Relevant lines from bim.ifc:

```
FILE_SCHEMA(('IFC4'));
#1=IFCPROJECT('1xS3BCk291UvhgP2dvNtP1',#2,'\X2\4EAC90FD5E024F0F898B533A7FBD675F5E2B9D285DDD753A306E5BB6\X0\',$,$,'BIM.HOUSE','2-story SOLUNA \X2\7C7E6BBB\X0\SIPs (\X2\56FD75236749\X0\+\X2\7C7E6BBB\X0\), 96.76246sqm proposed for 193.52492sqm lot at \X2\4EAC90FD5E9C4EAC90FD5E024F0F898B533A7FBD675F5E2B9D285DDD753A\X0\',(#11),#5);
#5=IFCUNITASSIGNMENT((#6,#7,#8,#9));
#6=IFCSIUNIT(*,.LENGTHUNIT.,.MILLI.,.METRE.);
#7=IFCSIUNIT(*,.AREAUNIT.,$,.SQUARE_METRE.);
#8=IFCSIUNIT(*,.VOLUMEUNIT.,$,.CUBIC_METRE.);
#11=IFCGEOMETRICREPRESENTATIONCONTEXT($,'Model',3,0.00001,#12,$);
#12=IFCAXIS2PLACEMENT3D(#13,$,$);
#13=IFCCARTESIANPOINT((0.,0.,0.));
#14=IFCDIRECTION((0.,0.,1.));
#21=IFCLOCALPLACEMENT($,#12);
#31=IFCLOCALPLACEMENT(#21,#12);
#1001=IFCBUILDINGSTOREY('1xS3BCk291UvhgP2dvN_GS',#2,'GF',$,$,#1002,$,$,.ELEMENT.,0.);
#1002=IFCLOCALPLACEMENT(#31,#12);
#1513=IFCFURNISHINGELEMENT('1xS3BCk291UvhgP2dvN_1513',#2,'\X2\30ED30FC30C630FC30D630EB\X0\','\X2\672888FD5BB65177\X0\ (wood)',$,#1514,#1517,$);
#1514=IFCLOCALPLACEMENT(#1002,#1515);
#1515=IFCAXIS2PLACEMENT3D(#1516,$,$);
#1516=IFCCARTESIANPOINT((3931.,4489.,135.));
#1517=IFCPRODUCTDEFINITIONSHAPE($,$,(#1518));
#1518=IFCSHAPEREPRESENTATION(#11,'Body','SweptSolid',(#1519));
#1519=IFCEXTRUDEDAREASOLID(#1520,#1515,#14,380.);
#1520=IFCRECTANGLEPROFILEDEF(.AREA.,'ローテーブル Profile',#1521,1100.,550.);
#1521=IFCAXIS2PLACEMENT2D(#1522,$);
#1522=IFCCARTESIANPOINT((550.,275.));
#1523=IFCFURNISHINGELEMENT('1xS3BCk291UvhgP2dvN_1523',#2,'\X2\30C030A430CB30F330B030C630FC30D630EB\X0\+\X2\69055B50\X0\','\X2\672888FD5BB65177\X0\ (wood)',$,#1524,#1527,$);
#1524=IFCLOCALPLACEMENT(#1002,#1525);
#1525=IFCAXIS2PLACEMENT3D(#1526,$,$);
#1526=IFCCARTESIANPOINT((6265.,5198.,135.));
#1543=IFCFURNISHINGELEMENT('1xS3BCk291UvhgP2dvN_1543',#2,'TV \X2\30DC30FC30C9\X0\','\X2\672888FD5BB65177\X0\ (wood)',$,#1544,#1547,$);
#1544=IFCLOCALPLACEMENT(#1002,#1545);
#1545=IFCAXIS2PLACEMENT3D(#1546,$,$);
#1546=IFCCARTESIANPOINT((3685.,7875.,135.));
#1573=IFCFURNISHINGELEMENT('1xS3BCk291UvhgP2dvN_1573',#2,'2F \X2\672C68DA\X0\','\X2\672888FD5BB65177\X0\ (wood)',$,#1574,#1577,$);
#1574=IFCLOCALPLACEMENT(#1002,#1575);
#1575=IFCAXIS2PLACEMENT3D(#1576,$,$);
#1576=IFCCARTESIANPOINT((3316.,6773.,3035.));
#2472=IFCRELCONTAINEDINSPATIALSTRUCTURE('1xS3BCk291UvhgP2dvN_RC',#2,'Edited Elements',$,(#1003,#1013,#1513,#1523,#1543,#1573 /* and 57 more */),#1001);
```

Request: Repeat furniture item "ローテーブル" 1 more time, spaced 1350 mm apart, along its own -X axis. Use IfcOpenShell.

```python
import ifcopenshell
import ifcopenshell.api.geometry
import ifcopenshell.api.root
import ifcopenshell.util.element
import ifcopenshell.util.placement

model = ifcopenshell.open("bim.ifc")


def reuse_history(source, copy):
    """copy_class also copies each property set's owner history, people and application; keep the originals."""
    for rel in copy.IsDefinedBy:
        if rel.is_a("IfcRelDefinesByProperties") and (history := rel.RelatingPropertyDefinition.OwnerHistory):
            rel.RelatingPropertyDefinition.OwnerHistory = source.OwnerHistory
            ifcopenshell.util.element.remove_deep2(model, history)


source = model.by_guid("1xS3BCk291UvhgP2dvN_1513")
base = ifcopenshell.util.placement.get_local_placement(source.ObjectPlacement)
step = -base[:3, 0] * 1350.0

for i in range(1, 2):
    copy = ifcopenshell.api.root.copy_class(model, product=source)
    copy.Representation = ifcopenshell.util.element.copy_deep(
        model, source.Representation, exclude=["IfcGeometricRepresentationContext", "IfcRepresentationMap"]
    )
    reuse_history(source, copy)
    matrix = base.copy()
    matrix[:3, 3] += i * step
    print("added at", matrix[:3, 3].round(3) + 0.0)
    ifcopenshell.api.geometry.edit_object_placement(model, product=copy, matrix=matrix, is_si=False)

model.write("bim_rev.ifc")
```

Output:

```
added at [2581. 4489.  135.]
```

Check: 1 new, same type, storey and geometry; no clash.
